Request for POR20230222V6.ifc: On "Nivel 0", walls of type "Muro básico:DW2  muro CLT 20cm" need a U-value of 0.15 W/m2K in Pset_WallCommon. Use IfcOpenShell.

First a look at what the model holds.

```python
import ifcopenshell
import ifcopenshell.util.element

model = ifcopenshell.open("POR20230222V6.ifc")
print(model.schema)
storey = next(s for s in model.by_type("IfcBuildingStorey") if s.Name == "Nivel 0")
walls = [e for e in ifcopenshell.util.element.get_decomposition(storey) if e.is_a("IfcWall")]
seen = {}
for e in walls:
    element_type = ifcopenshell.util.element.get_type(e)
    key = (element_type.Name if element_type != e and element_type else None, ifcopenshell.util.element.get_pset(e, "Pset_WallCommon", "ThermalTransmittance"))
    seen[key] = seen.get(key, 0) + 1
for (name, value), count in sorted(seen.items(), key=str):
    print(count, "x", name, "|", value)
```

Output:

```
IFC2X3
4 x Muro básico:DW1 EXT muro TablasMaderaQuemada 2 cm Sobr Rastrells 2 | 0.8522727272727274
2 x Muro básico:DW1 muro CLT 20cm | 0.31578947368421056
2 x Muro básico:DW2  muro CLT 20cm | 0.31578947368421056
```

```python
import ifcopenshell
import ifcopenshell.api.pset
import ifcopenshell.util.element

model = ifcopenshell.open("POR20230222V6.ifc")

storey = next(s for s in model.by_type("IfcBuildingStorey") if s.Name == "Nivel 0")
walls = [e for e in ifcopenshell.util.element.get_decomposition(storey) if e.is_a("IfcWall")]

count = 0
for e in walls:
    element_type = ifcopenshell.util.element.get_type(e)
    if element_type in (None, e) or element_type.Name != "Muro básico:DW2  muro CLT 20cm":
        continue
    # add_pset returns the element's existing set when there is one.
    pset = ifcopenshell.api.pset.add_pset(model, product=e, name="Pset_WallCommon")
    ifcopenshell.api.pset.edit_pset(model, pset=pset, properties={"ThermalTransmittance": 0.15})
    count += 1

print(count, "walls updated")

model.write("POR20230222V6_v2.ifc")
```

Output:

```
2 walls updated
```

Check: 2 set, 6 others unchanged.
